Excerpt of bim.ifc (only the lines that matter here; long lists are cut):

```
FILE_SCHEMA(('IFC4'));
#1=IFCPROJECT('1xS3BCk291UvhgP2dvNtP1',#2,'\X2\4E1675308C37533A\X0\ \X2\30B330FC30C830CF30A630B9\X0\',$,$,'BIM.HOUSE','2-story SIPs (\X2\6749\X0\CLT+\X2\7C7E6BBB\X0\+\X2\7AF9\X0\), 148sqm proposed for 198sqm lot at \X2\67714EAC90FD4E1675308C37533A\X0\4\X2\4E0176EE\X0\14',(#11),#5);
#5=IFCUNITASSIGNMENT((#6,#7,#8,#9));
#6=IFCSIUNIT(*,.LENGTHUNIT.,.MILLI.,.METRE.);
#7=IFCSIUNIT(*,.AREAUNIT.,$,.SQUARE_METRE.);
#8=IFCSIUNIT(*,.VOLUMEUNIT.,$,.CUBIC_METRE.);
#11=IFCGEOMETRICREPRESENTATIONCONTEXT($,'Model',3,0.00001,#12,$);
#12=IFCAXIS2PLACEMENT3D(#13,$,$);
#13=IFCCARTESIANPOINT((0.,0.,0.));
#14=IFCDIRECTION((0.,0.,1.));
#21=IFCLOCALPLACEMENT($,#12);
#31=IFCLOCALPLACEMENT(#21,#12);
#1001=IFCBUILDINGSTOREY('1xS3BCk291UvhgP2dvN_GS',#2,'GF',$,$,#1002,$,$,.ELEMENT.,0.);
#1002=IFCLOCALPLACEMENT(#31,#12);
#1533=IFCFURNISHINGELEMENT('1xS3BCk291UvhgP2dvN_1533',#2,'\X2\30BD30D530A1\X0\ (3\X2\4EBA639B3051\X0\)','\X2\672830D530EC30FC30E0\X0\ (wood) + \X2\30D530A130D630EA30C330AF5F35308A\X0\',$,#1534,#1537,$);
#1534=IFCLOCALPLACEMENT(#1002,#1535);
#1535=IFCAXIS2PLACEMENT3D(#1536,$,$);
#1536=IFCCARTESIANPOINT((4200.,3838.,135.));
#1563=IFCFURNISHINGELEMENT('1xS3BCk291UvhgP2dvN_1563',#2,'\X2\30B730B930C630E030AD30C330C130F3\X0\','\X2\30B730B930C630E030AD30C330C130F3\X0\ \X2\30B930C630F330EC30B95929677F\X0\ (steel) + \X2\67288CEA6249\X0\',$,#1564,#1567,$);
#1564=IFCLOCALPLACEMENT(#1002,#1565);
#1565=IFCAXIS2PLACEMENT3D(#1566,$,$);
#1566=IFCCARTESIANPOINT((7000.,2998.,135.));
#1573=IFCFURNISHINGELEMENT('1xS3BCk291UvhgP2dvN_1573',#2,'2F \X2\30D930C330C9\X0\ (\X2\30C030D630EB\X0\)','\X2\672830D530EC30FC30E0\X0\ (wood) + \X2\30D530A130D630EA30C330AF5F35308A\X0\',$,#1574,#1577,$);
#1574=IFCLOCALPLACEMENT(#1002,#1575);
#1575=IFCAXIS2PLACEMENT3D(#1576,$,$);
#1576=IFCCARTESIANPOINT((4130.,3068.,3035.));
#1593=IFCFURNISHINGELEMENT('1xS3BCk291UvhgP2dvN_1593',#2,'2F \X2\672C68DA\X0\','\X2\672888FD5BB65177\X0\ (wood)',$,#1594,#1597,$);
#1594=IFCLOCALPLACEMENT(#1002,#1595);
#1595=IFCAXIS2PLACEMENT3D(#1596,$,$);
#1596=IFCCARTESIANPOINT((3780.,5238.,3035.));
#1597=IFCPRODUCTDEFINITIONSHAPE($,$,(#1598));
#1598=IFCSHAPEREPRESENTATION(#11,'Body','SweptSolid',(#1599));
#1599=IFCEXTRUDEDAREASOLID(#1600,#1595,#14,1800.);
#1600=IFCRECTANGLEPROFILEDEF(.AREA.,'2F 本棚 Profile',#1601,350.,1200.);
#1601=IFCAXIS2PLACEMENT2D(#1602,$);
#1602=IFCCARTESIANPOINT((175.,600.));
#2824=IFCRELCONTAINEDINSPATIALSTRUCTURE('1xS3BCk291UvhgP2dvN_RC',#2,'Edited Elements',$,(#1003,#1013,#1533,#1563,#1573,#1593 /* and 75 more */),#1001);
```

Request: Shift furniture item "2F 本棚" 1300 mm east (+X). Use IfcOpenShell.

```python
import ifcopenshell
import ifcopenshell.api.geometry
import ifcopenshell.util.placement
import ifcopenshell.util.unit

model = ifcopenshell.open("bim.ifc")
unit_scale = ifcopenshell.util.unit.calculate_unit_scale(model)

item = model.by_guid("1xS3BCk291UvhgP2dvN_1593")
matrix = ifcopenshell.util.placement.get_local_placement(item.ObjectPlacement)
matrix[0, 3] += 1.3 / unit_scale
ifcopenshell.api.geometry.edit_object_placement(model, product=item, matrix=matrix, is_si=False)

print(ifcopenshell.util.placement.get_local_placement(item.ObjectPlacement).round(3) + 0.0)

model.write("bim-out.ifc")
```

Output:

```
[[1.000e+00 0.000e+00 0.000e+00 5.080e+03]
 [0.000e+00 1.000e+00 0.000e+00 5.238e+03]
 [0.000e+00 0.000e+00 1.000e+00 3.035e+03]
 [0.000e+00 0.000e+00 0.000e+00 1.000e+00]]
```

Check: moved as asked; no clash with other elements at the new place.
